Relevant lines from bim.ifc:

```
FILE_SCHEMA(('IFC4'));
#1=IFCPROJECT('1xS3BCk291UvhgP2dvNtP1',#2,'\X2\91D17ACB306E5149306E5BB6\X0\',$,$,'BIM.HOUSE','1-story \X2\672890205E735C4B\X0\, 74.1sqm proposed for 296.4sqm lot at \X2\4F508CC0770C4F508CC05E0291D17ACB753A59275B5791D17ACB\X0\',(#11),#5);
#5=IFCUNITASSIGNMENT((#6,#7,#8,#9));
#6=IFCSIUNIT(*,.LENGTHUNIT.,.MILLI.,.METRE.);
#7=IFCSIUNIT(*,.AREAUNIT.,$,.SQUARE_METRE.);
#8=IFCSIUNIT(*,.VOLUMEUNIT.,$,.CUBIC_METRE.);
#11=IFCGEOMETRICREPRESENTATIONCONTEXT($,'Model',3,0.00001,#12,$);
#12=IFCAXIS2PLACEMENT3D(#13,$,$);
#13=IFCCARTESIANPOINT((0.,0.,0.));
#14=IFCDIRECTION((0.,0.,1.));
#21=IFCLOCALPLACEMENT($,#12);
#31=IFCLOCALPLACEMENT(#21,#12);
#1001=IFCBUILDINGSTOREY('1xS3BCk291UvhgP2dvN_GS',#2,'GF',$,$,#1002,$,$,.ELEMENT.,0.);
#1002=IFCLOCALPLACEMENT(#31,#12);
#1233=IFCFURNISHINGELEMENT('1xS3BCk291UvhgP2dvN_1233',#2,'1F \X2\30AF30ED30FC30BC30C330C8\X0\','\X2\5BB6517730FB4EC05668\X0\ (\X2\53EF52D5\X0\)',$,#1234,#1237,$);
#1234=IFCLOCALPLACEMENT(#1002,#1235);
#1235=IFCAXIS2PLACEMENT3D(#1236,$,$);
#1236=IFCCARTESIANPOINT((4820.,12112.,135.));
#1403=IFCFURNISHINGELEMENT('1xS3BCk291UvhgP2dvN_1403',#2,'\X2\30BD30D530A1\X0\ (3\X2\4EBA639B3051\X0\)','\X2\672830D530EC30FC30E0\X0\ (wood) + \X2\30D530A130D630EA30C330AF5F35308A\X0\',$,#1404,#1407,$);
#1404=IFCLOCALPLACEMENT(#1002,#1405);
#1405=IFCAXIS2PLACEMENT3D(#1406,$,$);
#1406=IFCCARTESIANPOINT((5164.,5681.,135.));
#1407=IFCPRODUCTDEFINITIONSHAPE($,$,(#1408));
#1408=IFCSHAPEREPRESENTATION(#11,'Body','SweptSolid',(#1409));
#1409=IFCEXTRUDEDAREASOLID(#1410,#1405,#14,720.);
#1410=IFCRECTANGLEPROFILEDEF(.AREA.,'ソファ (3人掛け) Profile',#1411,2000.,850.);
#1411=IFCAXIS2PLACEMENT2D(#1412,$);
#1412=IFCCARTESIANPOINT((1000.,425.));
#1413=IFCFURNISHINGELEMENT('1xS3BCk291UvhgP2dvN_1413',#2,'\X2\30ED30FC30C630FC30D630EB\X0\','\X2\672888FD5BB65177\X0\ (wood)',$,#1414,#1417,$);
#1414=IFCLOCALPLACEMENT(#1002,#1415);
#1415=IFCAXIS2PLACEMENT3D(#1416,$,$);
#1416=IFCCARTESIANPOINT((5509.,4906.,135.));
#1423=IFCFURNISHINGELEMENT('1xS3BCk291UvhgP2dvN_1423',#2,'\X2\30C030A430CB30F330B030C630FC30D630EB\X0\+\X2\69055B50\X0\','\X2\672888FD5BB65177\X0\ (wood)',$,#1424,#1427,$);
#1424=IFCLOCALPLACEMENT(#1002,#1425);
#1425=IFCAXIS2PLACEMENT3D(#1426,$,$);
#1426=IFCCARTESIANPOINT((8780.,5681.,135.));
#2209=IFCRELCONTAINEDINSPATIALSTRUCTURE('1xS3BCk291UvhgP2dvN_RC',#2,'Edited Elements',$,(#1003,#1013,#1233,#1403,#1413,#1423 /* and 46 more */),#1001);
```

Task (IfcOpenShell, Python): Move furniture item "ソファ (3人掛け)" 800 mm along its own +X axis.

```python
import ifcopenshell
import ifcopenshell.api.geometry
import ifcopenshell.util.placement
import ifcopenshell.util.unit

model = ifcopenshell.open("bim.ifc")
unit_scale = ifcopenshell.util.unit.calculate_unit_scale(model)

item = model.by_guid("1xS3BCk291UvhgP2dvN_1403")
matrix = ifcopenshell.util.placement.get_local_placement(item.ObjectPlacement)
matrix[:3, 3] += matrix[:3, 0] * 0.8 / unit_scale
ifcopenshell.api.geometry.edit_object_placement(model, product=item, matrix=matrix, is_si=False)

print(ifcopenshell.util.placement.get_local_placement(item.ObjectPlacement).round(3) + 0.0)

model.write("bim_edited.ifc")
```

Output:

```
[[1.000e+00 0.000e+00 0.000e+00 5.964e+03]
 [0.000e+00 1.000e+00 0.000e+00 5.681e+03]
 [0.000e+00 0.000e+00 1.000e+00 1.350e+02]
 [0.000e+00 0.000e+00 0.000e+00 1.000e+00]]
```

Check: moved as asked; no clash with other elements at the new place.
